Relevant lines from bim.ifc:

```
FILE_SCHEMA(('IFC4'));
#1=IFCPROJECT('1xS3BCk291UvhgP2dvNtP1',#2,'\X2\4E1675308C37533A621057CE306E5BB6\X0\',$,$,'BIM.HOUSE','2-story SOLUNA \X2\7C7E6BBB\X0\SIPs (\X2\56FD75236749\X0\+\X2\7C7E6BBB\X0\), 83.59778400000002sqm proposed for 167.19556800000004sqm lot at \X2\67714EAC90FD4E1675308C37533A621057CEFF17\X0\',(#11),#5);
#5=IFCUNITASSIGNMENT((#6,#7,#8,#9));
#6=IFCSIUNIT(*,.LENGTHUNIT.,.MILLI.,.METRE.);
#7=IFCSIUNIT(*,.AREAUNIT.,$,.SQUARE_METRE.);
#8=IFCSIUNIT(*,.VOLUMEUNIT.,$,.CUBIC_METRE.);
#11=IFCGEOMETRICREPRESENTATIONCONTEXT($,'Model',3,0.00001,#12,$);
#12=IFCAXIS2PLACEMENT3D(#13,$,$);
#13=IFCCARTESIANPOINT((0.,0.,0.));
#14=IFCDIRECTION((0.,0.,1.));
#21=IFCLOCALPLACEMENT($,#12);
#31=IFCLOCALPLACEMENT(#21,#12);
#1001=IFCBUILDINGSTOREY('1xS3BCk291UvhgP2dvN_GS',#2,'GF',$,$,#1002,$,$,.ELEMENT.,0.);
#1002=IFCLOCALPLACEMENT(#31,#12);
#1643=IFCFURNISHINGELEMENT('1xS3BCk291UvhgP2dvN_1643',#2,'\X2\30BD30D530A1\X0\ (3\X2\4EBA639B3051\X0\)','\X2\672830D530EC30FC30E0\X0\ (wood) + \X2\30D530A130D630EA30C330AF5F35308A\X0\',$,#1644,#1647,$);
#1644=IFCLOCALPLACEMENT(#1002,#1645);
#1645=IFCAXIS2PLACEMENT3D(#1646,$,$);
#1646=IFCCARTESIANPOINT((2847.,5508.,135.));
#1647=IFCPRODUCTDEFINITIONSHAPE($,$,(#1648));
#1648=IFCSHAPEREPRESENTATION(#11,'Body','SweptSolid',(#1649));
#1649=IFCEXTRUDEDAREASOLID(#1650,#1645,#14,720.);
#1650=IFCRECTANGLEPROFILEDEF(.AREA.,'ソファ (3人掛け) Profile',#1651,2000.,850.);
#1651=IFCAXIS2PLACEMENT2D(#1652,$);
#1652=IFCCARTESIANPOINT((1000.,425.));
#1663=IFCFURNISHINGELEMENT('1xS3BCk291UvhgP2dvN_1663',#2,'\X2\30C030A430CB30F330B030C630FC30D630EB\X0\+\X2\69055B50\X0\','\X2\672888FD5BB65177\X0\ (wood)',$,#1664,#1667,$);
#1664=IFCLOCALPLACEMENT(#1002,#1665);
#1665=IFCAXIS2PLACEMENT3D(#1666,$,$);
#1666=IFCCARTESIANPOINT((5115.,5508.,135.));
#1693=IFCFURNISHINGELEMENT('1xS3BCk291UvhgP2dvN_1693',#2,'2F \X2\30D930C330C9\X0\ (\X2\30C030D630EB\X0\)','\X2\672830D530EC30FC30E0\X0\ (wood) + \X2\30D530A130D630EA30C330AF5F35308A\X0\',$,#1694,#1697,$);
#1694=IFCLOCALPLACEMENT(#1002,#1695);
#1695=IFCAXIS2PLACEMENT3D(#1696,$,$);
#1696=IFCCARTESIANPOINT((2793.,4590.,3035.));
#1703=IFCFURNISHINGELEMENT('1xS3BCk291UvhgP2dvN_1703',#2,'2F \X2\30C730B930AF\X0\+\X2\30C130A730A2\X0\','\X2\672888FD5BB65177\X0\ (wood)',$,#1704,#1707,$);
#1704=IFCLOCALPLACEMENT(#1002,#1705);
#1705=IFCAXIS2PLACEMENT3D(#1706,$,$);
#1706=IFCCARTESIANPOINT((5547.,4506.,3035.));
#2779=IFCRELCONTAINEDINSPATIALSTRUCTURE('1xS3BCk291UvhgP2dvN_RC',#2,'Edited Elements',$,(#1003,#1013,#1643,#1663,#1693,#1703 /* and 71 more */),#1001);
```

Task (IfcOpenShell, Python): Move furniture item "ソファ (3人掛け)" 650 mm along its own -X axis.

```python
import ifcopenshell
import ifcopenshell.api.geometry
import ifcopenshell.util.placement

model = ifcopenshell.open("bim.ifc")

item = model.by_guid("1xS3BCk291UvhgP2dvN_1643")
matrix = ifcopenshell.util.placement.get_local_placement(item.ObjectPlacement)
matrix[:3, 3] -= matrix[:3, 0] * 650.0
ifcopenshell.api.geometry.edit_object_placement(model, product=item, matrix=matrix, is_si=False)

print(ifcopenshell.util.placement.get_local_placement(item.ObjectPlacement).round(3) + 0.0)

model.write("bim_v2.ifc")
```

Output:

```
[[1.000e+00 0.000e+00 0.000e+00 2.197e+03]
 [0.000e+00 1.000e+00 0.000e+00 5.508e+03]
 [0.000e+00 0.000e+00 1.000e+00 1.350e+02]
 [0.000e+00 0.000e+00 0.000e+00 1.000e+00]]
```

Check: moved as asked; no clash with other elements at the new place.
